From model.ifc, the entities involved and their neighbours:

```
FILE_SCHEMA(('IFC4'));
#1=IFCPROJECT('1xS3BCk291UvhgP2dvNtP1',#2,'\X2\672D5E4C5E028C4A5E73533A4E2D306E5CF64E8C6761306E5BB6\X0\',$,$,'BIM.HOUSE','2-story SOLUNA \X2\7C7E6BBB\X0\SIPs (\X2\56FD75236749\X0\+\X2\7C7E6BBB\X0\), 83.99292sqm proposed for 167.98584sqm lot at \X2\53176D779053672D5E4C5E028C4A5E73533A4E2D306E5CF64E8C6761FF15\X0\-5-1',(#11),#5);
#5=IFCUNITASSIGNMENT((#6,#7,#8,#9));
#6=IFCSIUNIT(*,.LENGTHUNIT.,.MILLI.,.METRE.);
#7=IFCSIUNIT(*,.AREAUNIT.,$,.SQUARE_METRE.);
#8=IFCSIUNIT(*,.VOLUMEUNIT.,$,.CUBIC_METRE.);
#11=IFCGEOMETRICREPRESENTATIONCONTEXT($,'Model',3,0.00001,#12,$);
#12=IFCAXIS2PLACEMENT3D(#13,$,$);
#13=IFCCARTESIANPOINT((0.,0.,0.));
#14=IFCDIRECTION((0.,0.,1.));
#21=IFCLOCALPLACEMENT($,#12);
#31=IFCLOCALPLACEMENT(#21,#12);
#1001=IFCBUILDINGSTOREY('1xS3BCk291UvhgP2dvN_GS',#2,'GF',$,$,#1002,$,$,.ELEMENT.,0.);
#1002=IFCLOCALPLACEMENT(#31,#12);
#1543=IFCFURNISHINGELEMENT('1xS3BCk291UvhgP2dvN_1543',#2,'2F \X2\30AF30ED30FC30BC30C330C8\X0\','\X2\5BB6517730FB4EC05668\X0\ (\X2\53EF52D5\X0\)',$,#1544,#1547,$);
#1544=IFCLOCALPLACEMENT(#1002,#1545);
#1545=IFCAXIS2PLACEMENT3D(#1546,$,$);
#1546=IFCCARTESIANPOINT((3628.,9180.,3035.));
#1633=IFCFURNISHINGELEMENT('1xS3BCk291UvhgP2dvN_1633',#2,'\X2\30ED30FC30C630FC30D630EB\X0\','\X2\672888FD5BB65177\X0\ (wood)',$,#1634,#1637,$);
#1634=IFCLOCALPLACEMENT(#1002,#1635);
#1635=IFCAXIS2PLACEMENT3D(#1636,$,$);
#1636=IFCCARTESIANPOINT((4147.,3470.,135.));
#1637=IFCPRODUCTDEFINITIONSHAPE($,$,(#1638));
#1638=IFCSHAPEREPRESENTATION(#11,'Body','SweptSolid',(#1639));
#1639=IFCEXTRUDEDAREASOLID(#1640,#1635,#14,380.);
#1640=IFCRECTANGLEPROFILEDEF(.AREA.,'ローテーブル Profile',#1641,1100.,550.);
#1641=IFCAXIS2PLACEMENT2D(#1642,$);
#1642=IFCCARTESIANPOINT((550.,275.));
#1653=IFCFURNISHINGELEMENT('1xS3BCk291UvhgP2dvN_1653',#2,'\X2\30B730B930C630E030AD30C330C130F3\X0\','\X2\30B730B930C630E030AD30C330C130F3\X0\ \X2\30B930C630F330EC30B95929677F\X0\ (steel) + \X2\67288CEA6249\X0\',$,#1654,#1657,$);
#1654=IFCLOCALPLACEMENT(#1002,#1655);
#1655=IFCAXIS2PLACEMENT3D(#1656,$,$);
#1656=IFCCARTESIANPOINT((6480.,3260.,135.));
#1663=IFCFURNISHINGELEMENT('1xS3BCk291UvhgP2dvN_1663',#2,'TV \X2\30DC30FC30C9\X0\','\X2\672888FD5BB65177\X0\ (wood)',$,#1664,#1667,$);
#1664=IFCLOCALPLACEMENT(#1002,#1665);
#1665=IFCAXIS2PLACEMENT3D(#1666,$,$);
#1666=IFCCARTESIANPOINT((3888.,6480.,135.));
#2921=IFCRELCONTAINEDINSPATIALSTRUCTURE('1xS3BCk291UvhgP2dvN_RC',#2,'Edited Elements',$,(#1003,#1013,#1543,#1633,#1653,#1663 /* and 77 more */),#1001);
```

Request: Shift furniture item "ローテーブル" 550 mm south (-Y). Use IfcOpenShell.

```python
import ifcopenshell
import ifcopenshell.api.geometry
import ifcopenshell.util.placement

model = ifcopenshell.open("model.ifc")

item = model.by_guid("1xS3BCk291UvhgP2dvN_1633")
matrix = ifcopenshell.util.placement.get_local_placement(item.ObjectPlacement)
matrix[1, 3] -= 550.0
ifcopenshell.api.geometry.edit_object_placement(model, product=item, matrix=matrix, is_si=False)

print(ifcopenshell.util.placement.get_local_placement(item.ObjectPlacement).round(3) + 0.0)

model.write("model_updated.ifc")
```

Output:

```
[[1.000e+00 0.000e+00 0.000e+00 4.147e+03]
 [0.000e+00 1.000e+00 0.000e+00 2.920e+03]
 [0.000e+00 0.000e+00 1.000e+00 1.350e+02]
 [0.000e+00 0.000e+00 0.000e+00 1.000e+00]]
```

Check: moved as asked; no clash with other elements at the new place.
